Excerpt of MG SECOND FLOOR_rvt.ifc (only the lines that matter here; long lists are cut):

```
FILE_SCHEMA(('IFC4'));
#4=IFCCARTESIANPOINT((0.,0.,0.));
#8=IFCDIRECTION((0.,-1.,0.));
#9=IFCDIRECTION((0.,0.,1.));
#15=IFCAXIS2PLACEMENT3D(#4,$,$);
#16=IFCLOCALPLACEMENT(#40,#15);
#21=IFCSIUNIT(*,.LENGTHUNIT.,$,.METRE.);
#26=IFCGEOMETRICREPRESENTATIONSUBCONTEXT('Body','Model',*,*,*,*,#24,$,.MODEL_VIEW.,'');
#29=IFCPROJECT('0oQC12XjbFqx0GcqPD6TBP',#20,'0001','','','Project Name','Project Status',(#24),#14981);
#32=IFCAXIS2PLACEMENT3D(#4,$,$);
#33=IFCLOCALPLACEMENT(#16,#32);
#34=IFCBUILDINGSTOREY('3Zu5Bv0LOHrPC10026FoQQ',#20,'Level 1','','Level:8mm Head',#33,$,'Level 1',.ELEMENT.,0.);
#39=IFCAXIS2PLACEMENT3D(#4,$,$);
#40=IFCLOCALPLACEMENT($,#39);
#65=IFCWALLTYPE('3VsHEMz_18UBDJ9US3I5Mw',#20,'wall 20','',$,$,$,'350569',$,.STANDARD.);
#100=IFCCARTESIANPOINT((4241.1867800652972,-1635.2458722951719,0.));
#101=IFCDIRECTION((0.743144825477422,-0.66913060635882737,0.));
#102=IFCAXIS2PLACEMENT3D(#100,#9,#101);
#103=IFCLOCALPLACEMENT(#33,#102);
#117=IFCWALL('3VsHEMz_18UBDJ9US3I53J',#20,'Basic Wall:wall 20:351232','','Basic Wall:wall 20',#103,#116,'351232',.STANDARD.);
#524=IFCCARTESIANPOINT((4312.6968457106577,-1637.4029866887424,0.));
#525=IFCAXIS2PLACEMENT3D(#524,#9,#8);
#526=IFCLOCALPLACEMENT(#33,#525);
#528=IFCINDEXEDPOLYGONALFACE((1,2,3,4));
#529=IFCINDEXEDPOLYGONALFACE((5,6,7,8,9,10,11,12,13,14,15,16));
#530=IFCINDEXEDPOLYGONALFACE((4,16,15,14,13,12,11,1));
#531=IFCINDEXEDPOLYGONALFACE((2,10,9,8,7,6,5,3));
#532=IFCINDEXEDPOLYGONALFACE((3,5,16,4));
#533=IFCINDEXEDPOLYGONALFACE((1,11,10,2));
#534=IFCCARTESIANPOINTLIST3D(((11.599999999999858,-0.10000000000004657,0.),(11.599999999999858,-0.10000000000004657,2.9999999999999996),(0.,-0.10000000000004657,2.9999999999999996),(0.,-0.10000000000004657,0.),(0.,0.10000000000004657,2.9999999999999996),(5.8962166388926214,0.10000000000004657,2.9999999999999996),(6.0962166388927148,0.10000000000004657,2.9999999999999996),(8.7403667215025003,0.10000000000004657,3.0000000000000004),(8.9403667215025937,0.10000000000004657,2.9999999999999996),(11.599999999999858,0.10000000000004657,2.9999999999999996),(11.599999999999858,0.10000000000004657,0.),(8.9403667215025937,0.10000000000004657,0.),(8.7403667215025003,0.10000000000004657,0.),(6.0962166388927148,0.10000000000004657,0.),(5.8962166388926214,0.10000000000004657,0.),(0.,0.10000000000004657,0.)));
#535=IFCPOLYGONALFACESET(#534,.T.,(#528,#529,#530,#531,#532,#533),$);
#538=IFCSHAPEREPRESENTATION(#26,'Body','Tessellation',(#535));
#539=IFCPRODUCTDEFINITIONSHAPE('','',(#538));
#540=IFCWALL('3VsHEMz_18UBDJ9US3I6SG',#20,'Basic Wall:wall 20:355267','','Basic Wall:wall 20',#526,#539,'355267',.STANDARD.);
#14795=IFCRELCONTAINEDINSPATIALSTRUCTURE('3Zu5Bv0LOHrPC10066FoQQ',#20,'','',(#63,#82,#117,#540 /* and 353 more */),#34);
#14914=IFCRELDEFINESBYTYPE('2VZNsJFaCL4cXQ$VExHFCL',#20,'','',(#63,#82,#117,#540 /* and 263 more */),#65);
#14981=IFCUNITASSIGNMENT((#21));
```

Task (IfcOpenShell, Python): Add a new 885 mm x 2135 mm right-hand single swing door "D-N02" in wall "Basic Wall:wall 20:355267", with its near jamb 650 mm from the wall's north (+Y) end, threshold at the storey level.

```python
import numpy as np
import ifcopenshell
import ifcopenshell.api.feature
import ifcopenshell.api.geometry
import ifcopenshell.api.root
import ifcopenshell.api.spatial
import ifcopenshell.geom
import ifcopenshell.util.element
import ifcopenshell.util.placement
import ifcopenshell.util.representation
import ifcopenshell.util.shape
import ifcopenshell.util.unit

model = ifcopenshell.open("MG SECOND FLOOR_rvt.ifc")
unit_scale = ifcopenshell.util.unit.calculate_unit_scale(model)
settings = ifcopenshell.geom.settings()


def volume(element):
    """Net volume in cubic metres, openings subtracted."""
    shape = ifcopenshell.geom.create_shape(settings, element)
    return ifcopenshell.util.shape.get_volume(shape.geometry)


wall = model.by_guid("3VsHEMz_18UBDJ9US3I6SG")
storey = ifcopenshell.util.element.get_container(wall, ifc_class="IfcBuildingStorey")
context = ifcopenshell.util.representation.get_context(model, "Model", "Body", "MODEL_VIEW")
before = volume(wall)

width, height, from_end, sill = 0.885, 2.135, 0.65, 0.0  # metres

# The wall runs along its own X axis, and the end named is its -X end.
wall_shape = ifcopenshell.geom.create_shape(settings, wall)
x, y, z = ifcopenshell.util.shape.get_vertices(wall_shape.geometry).T
start = x.min() + from_end
face, thickness = float(y.min()), float(y.max() - y.min())
wall_matrix = ifcopenshell.util.placement.get_local_placement(wall.ObjectPlacement)
level = ifcopenshell.util.placement.get_local_placement(storey.ObjectPlacement)[2, 3]


def in_wall(x, y):
    """Placement at x, y metres in the wall's axes, at sill height."""
    matrix = wall_matrix.copy()
    matrix[:, 3] = wall_matrix @ np.array([x / unit_scale, y / unit_scale, 0.0, 1.0])
    matrix[2, 3] = level + sill / unit_scale
    return matrix


# Opening: a box that overshoots both wall faces by 50 mm.
opening = ifcopenshell.api.root.create_entity(model, ifc_class="IfcOpeningElement", predefined_type="OPENING")
box = ifcopenshell.api.geometry.add_wall_representation(
    model, context=context, length=width, height=height, thickness=thickness + 0.1
)
ifcopenshell.api.geometry.assign_representation(model, product=opening, representation=box)
ifcopenshell.api.geometry.edit_object_placement(model, product=opening, matrix=in_wall(start, face - 0.05), is_si=False)
ifcopenshell.api.feature.add_feature(model, feature=opening, element=wall)

door = ifcopenshell.api.root.create_entity(model, ifc_class="IfcDoor", name="D-N02", predefined_type="DOOR")
door.OverallWidth, door.OverallHeight = width / unit_scale, height / unit_scale
door.OperationType = "SINGLE_SWING_RIGHT"
body = ifcopenshell.api.geometry.add_door_representation(
    model,
    context=context,
    overall_width=door.OverallWidth,
    overall_height=door.OverallHeight,
    operation_type="SINGLE_SWING_RIGHT",
    lining_properties={"LiningDepth": thickness / unit_scale, "ThresholdDepth": thickness / unit_scale},
)
ifcopenshell.api.geometry.assign_representation(model, product=door, representation=body)
ifcopenshell.api.spatial.assign_container(model, products=[door], relating_structure=storey)
ifcopenshell.api.feature.add_filling(model, opening=opening, element=door)

# The lining spans the wall, so the door starts at the wall face.
ifcopenshell.api.geometry.edit_object_placement(model, product=door, matrix=in_wall(start, face), is_si=False)

after = volume(wall)

print(f"wall volume {before:.3f} -> {after:.3f} m3")

model.write("MG SECOND FLOOR_rvt_updated.ifc")
```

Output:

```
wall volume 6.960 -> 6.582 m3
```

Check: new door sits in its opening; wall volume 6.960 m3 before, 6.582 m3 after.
